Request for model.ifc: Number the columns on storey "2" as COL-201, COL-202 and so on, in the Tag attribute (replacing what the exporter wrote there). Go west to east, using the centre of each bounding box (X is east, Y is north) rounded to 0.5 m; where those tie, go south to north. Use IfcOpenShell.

First a look at what the model holds.

```python
import ifcopenshell
import ifcopenshell.util.element
import ifcopenshell.util.placement

model = ifcopenshell.open("model.ifc")
print(model.schema)
storey = next(s for s in model.by_type("IfcBuildingStorey") if s.Name == "2")
columns = [e for e in ifcopenshell.util.element.get_decomposition(storey) if e.is_a("IfcColumn")]
for e in sorted(columns, key=lambda e: e.id()):
    origin = ifcopenshell.util.placement.get_local_placement(e.ObjectPlacement)[:3, 3]
    print(e.id(), e.Tag, e.Name, origin.round(2) + 0.0, sep=" | ")
```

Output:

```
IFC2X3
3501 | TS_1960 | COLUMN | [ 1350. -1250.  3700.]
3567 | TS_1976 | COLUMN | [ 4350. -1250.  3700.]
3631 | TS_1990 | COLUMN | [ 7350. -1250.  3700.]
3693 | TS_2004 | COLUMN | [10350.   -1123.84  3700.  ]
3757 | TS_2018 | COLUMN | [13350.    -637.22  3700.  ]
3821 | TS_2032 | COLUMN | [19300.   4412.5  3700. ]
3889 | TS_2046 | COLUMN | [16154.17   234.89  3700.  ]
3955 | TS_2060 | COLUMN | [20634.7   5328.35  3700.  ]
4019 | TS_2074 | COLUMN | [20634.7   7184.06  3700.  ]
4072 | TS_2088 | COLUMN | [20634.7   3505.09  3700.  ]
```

```python
import ifcopenshell
import ifcopenshell.geom
import ifcopenshell.util.element
import ifcopenshell.util.shape

model = ifcopenshell.open("model.ifc")
settings = ifcopenshell.geom.settings()
settings.set("use-world-coords", True)


def centre(element):
    shape = ifcopenshell.geom.create_shape(settings, element)
    return ifcopenshell.util.shape.get_bbox_centroid(shape.geometry)


storey = next(s for s in model.by_type("IfcBuildingStorey") if s.Name == "2")
columns = [e for e in ifcopenshell.util.element.get_decomposition(storey) if e.is_a("IfcColumn")]

# Insertion points can sit at a corner or the storey origin, so sort by the geometry (in metres).
centres = {e: centre(e) for e in columns}
columns.sort(key=lambda e: (round(centres[e][0] / 0.5), centres[e][1]))

for i, e in enumerate(columns, start=1):
    number = f"COL-2{i:02d}"
    e.Tag = number
    print(e.id(), number)

model.write("model_v2.ifc")
```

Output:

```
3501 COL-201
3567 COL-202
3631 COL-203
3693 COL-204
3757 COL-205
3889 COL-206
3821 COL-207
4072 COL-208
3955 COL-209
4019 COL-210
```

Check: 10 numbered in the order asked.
